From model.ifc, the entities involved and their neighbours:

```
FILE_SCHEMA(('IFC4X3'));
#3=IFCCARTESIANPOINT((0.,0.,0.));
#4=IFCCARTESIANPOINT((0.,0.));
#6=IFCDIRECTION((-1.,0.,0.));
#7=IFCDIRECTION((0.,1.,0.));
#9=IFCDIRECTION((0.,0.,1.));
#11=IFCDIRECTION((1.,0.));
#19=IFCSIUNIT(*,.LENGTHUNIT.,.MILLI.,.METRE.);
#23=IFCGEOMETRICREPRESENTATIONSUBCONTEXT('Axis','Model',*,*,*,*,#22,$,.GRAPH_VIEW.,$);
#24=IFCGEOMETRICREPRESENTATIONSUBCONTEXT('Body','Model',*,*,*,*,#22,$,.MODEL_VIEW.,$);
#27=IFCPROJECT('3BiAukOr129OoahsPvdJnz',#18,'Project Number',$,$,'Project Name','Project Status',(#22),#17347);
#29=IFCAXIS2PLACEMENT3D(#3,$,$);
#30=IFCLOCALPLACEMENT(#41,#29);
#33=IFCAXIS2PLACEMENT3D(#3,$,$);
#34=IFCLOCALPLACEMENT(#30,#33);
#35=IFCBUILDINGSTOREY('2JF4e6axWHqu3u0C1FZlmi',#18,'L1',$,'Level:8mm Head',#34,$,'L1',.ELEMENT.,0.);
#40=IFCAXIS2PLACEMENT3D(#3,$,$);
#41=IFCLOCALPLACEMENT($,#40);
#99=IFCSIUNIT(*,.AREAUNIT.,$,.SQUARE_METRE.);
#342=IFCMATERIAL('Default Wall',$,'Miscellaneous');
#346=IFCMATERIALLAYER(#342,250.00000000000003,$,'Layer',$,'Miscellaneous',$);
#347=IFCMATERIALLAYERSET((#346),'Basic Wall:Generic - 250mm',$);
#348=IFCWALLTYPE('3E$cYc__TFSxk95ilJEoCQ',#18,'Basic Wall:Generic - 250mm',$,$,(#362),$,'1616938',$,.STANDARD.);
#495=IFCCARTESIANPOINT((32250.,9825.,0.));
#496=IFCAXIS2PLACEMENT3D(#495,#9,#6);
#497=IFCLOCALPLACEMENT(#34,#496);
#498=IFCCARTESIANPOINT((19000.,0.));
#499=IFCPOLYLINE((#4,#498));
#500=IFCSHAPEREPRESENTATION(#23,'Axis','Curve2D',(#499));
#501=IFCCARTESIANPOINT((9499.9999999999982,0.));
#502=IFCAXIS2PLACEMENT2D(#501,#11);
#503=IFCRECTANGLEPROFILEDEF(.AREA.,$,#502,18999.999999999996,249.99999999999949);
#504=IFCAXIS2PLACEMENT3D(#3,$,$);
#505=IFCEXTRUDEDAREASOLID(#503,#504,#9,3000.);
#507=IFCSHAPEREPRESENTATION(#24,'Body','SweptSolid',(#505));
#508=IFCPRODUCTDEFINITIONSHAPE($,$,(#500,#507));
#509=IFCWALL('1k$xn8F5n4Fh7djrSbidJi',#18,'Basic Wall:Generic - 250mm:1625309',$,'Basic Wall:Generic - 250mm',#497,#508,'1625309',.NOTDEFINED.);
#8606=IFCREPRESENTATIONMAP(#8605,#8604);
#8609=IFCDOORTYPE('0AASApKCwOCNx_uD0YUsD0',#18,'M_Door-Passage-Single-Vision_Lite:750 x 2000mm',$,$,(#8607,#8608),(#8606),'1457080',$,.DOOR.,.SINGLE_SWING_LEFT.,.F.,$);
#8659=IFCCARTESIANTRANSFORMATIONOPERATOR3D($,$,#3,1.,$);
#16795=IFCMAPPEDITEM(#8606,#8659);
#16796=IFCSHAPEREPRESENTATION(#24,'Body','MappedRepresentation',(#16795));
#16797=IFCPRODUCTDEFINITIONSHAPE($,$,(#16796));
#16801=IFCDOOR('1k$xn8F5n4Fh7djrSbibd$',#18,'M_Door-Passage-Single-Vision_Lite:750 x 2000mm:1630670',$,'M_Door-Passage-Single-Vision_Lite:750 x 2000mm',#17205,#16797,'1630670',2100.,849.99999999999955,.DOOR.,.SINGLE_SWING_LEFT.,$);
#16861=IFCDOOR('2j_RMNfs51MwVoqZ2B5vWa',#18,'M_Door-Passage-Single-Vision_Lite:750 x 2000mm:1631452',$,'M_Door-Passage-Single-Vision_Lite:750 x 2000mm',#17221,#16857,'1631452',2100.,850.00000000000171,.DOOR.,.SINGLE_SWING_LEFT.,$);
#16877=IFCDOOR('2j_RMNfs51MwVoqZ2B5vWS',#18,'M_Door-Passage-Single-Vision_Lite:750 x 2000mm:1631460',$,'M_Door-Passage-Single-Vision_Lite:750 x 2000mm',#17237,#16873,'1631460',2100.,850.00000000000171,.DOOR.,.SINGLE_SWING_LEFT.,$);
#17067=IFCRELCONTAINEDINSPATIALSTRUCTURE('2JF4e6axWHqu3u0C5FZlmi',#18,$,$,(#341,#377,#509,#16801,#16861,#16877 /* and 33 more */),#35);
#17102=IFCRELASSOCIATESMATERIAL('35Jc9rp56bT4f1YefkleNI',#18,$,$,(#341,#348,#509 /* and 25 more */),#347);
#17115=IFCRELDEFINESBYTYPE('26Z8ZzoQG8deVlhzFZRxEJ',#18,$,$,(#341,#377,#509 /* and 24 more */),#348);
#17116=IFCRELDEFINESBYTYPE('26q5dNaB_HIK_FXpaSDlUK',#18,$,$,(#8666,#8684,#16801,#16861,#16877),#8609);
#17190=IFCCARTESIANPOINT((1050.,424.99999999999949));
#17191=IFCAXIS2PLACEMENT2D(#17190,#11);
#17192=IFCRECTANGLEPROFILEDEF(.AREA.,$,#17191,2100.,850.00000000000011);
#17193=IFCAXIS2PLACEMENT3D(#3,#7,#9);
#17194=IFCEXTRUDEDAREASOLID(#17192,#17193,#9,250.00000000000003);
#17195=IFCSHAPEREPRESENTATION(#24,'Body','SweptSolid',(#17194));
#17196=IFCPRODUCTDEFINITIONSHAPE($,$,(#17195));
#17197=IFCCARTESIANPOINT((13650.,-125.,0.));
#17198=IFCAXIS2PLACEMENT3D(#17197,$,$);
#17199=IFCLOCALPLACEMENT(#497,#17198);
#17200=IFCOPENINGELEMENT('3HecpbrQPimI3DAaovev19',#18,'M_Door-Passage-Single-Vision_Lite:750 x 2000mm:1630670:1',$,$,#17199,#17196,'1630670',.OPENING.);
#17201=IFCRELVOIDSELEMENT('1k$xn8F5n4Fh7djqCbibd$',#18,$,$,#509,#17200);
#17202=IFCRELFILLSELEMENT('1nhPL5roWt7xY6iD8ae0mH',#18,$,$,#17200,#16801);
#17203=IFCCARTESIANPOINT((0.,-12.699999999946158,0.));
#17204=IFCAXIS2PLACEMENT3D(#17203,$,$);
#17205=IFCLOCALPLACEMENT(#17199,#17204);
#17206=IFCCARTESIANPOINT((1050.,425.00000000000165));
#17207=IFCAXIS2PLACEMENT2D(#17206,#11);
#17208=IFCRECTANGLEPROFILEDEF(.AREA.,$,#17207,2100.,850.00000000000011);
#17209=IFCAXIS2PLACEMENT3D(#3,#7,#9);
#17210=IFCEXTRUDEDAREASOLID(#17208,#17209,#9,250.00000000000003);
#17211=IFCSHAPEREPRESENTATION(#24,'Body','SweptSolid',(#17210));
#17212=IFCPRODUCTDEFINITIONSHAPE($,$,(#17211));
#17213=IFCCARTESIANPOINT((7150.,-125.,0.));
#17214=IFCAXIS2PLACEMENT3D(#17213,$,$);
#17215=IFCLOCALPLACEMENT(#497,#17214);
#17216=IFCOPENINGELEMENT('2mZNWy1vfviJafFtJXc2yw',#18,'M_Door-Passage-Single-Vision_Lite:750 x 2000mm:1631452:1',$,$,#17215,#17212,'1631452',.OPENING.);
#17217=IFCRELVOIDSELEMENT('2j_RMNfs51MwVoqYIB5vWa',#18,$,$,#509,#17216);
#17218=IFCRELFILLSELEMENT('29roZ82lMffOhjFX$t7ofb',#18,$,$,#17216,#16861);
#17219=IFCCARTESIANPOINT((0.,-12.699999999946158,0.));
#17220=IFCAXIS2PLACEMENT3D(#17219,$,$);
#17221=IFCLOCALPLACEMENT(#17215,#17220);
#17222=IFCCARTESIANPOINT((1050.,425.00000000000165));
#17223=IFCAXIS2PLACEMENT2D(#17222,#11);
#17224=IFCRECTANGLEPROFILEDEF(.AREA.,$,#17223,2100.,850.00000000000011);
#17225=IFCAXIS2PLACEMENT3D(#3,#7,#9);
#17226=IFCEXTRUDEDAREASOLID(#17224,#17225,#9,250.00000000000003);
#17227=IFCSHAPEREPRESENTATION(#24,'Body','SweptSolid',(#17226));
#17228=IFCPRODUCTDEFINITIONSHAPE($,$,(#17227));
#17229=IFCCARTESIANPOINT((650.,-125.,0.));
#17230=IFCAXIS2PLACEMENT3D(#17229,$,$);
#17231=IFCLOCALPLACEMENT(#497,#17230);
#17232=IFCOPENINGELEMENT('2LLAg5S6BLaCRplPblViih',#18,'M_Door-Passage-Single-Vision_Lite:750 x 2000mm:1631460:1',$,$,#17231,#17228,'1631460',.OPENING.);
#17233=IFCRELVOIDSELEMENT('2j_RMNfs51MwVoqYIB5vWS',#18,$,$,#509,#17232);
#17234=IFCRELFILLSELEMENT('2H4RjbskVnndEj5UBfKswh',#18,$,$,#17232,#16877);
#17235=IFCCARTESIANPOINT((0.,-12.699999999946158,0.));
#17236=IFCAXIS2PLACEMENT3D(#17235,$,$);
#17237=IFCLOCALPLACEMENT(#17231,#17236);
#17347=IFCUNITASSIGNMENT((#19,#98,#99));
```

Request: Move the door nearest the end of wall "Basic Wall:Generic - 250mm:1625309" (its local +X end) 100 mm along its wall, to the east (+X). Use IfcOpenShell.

```python
import ifcopenshell
import ifcopenshell.api.geometry
import ifcopenshell.util.placement
import ifcopenshell.util.unit

model = ifcopenshell.open("model.ifc")
unit_scale = ifcopenshell.util.unit.calculate_unit_scale(model)

door = model.by_id(16801)
opening = door.FillsVoids[0].RelatingOpeningElement
wall = opening.VoidsElements[0].RelatingBuildingElement

wall_matrix = ifcopenshell.util.placement.get_local_placement(wall.ObjectPlacement)
shift = wall_matrix[:3, 0] * -0.1 / unit_scale
before = ifcopenshell.util.placement.get_local_placement(door.ObjectPlacement)[:3, 3].copy()

# The door is placed relative to its opening, so it follows when the opening moves.
matrix = ifcopenshell.util.placement.get_local_placement(opening.ObjectPlacement)
matrix[:3, 3] += shift
ifcopenshell.api.geometry.edit_object_placement(
    model, product=opening, matrix=matrix, is_si=False, should_transform_children=True
)

after = ifcopenshell.util.placement.get_local_placement(door.ObjectPlacement)[:3, 3]
print("door moved by", (after - before).round(3) + 0.0)

model.write("model-out.ifc")
```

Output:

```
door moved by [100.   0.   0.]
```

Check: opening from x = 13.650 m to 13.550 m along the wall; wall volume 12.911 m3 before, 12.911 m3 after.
